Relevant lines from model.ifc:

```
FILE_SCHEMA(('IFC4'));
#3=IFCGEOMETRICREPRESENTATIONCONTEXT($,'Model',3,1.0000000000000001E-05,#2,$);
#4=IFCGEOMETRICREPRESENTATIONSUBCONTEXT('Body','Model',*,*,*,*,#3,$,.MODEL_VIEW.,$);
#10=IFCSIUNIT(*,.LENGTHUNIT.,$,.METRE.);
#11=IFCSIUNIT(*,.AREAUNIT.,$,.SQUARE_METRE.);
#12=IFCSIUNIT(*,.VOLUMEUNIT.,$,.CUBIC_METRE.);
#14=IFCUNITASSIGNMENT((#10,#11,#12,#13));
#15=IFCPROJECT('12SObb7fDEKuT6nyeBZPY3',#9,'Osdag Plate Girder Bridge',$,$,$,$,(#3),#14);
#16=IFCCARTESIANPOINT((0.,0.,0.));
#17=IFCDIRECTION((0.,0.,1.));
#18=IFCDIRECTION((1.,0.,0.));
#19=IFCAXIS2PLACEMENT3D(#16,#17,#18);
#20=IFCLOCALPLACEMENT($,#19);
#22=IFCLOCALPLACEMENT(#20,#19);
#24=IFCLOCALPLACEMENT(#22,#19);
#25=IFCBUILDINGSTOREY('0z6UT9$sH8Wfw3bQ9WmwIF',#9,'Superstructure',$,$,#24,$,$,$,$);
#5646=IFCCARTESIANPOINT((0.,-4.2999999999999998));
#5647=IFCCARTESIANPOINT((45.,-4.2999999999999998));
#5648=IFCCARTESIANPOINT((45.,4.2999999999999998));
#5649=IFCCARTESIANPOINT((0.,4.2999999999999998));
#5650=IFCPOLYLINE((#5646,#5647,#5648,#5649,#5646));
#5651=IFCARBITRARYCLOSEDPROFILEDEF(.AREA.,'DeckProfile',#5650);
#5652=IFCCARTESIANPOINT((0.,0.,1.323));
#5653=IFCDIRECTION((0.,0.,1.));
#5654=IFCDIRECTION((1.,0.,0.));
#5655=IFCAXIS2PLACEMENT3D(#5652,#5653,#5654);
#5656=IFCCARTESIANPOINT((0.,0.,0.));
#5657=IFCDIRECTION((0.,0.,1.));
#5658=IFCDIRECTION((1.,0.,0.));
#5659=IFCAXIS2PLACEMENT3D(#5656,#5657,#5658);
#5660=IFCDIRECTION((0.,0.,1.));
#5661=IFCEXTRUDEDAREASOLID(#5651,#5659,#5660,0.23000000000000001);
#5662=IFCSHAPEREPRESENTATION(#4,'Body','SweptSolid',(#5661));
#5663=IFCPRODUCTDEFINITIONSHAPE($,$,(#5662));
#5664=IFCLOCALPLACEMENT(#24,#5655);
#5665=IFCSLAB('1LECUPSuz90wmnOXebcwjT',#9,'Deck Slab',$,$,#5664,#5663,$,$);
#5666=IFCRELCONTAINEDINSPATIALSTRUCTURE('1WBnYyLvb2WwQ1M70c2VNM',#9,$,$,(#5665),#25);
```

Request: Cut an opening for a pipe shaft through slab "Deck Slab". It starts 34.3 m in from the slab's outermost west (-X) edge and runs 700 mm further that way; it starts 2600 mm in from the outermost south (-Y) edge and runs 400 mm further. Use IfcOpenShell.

```python
import numpy as np
import ifcopenshell
import ifcopenshell.api.feature
import ifcopenshell.api.geometry
import ifcopenshell.api.root
import ifcopenshell.geom
import ifcopenshell.util.placement
import ifcopenshell.util.representation
import ifcopenshell.util.shape
import ifcopenshell.util.unit

model = ifcopenshell.open("model.ifc")
unit_scale = ifcopenshell.util.unit.calculate_unit_scale(model)
settings = ifcopenshell.geom.settings()


def volume(element):
    """Net volume in cubic metres, openings subtracted."""
    shape = ifcopenshell.geom.create_shape(settings, element)
    return ifcopenshell.util.shape.get_volume(shape.geometry)


slab = model.by_id(5665)
before = volume(slab)

# Extent in the slab's own axes, in metres. The edges named are its -X and -Y sides.
slab_shape = ifcopenshell.geom.create_shape(settings, slab)
vertices = ifcopenshell.util.shape.get_vertices(slab_shape.geometry)
x_min, y_min, bottom = vertices.min(axis=0)
top = vertices[:, 2].max()

opening = ifcopenshell.api.root.create_entity(model, ifc_class="IfcOpeningElement", name="Pipe shaft opening", predefined_type="OPENING")
context = ifcopenshell.util.representation.get_context(model, "Model", "Body", "MODEL_VIEW")
width, depth = 0.7, 0.4
outline = [(0.0, 0.0), (width, 0.0), (width, depth), (0.0, depth), (0.0, 0.0)]
# Overshoot both faces by 50 mm so the cut is clean.
shape = ifcopenshell.api.geometry.add_slab_representation(
    model, context=context, depth=top - bottom + 0.1, polyline=outline
)
ifcopenshell.api.geometry.assign_representation(model, product=opening, representation=shape)

matrix = ifcopenshell.util.placement.get_local_placement(slab.ObjectPlacement)
matrix[:, 3] = matrix @ np.append(np.array([x_min + 34.3, y_min + 2.6, bottom - 0.05]) / unit_scale, 1.0)
ifcopenshell.api.geometry.edit_object_placement(model, product=opening, matrix=matrix, is_si=False)
ifcopenshell.api.feature.add_feature(model, feature=opening, element=slab)

after = volume(slab)

print(f"slab volume {before:.3f} -> {after:.3f} m3")

model.write("model_v2.ifc")
```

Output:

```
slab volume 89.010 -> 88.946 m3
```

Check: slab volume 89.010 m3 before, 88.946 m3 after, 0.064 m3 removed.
